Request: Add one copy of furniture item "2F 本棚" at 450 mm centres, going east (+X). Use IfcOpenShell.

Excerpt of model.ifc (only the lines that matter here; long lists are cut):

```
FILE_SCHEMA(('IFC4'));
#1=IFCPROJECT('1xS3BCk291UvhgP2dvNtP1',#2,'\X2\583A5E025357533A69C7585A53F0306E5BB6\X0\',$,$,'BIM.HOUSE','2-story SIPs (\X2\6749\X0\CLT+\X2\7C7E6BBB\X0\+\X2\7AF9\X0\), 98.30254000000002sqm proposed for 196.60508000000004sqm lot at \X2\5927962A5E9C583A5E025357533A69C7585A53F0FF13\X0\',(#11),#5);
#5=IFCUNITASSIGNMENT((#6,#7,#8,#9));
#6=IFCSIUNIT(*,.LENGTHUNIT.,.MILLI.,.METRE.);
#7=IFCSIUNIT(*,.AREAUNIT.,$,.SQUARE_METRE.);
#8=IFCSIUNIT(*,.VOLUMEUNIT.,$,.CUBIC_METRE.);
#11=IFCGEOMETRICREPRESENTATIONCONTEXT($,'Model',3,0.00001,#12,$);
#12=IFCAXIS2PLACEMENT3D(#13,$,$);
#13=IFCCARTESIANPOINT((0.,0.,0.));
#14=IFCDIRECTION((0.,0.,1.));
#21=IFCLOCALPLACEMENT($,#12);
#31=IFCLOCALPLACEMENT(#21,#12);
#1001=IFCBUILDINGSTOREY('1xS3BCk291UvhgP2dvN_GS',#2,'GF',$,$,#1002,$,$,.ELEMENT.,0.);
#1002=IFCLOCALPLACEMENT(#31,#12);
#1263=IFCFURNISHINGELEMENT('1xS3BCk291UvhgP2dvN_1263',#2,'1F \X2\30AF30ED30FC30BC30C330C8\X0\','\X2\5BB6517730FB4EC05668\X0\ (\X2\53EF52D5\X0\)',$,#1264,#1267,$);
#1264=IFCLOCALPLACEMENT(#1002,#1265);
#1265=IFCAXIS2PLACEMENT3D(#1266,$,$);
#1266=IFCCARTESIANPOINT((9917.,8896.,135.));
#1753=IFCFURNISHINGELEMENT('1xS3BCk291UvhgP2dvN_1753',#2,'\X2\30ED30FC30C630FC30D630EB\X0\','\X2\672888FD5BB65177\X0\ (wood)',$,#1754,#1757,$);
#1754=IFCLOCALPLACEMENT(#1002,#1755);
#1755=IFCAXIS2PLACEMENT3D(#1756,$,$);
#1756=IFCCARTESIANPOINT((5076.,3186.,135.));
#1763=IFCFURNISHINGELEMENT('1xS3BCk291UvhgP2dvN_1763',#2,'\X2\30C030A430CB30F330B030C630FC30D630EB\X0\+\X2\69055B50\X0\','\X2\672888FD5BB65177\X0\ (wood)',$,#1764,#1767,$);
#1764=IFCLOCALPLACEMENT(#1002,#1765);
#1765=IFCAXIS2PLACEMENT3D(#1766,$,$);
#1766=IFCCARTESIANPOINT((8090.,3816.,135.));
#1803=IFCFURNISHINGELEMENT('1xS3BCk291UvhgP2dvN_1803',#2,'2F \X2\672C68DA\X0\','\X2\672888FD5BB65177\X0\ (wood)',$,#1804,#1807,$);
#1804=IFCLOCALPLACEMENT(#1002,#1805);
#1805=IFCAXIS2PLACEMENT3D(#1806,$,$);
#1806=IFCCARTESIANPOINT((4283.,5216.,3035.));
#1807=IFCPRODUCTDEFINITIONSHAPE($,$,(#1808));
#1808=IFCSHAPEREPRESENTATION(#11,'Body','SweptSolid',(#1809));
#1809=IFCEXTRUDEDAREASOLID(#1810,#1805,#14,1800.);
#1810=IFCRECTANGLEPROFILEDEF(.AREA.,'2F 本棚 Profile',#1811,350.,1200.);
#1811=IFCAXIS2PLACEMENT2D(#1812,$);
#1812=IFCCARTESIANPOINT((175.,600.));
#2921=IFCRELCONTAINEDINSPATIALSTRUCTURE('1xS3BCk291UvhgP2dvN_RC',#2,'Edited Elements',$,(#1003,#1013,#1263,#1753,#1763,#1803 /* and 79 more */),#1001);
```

```python
import numpy as np
import ifcopenshell
import ifcopenshell.api.geometry
import ifcopenshell.api.root
import ifcopenshell.util.element
import ifcopenshell.util.placement
import ifcopenshell.util.unit

model = ifcopenshell.open("model.ifc")
unit_scale = ifcopenshell.util.unit.calculate_unit_scale(model)


def reuse_history(source, copy):
    """copy_class also copies each property set's owner history, people and application; keep the originals."""
    for rel in copy.IsDefinedBy:
        if rel.is_a("IfcRelDefinesByProperties") and (history := rel.RelatingPropertyDefinition.OwnerHistory):
            rel.RelatingPropertyDefinition.OwnerHistory = source.OwnerHistory
            ifcopenshell.util.element.remove_deep2(model, history)


source = model.by_id(1803)
base = ifcopenshell.util.placement.get_local_placement(source.ObjectPlacement)
step = np.array([1.0, 0.0, 0.0]) * 0.45 / unit_scale

for i in range(1, 2):
    copy = ifcopenshell.api.root.copy_class(model, product=source)
    copy.Representation = ifcopenshell.util.element.copy_deep(
        model, source.Representation, exclude=["IfcGeometricRepresentationContext", "IfcRepresentationMap"]
    )
    reuse_history(source, copy)
    matrix = base.copy()
    matrix[:3, 3] += i * step
    print("added at", matrix[:3, 3].round(3) + 0.0)
    ifcopenshell.api.geometry.edit_object_placement(model, product=copy, matrix=matrix, is_si=False)

model.write("model_rev.ifc")
```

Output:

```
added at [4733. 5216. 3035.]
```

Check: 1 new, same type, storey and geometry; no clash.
